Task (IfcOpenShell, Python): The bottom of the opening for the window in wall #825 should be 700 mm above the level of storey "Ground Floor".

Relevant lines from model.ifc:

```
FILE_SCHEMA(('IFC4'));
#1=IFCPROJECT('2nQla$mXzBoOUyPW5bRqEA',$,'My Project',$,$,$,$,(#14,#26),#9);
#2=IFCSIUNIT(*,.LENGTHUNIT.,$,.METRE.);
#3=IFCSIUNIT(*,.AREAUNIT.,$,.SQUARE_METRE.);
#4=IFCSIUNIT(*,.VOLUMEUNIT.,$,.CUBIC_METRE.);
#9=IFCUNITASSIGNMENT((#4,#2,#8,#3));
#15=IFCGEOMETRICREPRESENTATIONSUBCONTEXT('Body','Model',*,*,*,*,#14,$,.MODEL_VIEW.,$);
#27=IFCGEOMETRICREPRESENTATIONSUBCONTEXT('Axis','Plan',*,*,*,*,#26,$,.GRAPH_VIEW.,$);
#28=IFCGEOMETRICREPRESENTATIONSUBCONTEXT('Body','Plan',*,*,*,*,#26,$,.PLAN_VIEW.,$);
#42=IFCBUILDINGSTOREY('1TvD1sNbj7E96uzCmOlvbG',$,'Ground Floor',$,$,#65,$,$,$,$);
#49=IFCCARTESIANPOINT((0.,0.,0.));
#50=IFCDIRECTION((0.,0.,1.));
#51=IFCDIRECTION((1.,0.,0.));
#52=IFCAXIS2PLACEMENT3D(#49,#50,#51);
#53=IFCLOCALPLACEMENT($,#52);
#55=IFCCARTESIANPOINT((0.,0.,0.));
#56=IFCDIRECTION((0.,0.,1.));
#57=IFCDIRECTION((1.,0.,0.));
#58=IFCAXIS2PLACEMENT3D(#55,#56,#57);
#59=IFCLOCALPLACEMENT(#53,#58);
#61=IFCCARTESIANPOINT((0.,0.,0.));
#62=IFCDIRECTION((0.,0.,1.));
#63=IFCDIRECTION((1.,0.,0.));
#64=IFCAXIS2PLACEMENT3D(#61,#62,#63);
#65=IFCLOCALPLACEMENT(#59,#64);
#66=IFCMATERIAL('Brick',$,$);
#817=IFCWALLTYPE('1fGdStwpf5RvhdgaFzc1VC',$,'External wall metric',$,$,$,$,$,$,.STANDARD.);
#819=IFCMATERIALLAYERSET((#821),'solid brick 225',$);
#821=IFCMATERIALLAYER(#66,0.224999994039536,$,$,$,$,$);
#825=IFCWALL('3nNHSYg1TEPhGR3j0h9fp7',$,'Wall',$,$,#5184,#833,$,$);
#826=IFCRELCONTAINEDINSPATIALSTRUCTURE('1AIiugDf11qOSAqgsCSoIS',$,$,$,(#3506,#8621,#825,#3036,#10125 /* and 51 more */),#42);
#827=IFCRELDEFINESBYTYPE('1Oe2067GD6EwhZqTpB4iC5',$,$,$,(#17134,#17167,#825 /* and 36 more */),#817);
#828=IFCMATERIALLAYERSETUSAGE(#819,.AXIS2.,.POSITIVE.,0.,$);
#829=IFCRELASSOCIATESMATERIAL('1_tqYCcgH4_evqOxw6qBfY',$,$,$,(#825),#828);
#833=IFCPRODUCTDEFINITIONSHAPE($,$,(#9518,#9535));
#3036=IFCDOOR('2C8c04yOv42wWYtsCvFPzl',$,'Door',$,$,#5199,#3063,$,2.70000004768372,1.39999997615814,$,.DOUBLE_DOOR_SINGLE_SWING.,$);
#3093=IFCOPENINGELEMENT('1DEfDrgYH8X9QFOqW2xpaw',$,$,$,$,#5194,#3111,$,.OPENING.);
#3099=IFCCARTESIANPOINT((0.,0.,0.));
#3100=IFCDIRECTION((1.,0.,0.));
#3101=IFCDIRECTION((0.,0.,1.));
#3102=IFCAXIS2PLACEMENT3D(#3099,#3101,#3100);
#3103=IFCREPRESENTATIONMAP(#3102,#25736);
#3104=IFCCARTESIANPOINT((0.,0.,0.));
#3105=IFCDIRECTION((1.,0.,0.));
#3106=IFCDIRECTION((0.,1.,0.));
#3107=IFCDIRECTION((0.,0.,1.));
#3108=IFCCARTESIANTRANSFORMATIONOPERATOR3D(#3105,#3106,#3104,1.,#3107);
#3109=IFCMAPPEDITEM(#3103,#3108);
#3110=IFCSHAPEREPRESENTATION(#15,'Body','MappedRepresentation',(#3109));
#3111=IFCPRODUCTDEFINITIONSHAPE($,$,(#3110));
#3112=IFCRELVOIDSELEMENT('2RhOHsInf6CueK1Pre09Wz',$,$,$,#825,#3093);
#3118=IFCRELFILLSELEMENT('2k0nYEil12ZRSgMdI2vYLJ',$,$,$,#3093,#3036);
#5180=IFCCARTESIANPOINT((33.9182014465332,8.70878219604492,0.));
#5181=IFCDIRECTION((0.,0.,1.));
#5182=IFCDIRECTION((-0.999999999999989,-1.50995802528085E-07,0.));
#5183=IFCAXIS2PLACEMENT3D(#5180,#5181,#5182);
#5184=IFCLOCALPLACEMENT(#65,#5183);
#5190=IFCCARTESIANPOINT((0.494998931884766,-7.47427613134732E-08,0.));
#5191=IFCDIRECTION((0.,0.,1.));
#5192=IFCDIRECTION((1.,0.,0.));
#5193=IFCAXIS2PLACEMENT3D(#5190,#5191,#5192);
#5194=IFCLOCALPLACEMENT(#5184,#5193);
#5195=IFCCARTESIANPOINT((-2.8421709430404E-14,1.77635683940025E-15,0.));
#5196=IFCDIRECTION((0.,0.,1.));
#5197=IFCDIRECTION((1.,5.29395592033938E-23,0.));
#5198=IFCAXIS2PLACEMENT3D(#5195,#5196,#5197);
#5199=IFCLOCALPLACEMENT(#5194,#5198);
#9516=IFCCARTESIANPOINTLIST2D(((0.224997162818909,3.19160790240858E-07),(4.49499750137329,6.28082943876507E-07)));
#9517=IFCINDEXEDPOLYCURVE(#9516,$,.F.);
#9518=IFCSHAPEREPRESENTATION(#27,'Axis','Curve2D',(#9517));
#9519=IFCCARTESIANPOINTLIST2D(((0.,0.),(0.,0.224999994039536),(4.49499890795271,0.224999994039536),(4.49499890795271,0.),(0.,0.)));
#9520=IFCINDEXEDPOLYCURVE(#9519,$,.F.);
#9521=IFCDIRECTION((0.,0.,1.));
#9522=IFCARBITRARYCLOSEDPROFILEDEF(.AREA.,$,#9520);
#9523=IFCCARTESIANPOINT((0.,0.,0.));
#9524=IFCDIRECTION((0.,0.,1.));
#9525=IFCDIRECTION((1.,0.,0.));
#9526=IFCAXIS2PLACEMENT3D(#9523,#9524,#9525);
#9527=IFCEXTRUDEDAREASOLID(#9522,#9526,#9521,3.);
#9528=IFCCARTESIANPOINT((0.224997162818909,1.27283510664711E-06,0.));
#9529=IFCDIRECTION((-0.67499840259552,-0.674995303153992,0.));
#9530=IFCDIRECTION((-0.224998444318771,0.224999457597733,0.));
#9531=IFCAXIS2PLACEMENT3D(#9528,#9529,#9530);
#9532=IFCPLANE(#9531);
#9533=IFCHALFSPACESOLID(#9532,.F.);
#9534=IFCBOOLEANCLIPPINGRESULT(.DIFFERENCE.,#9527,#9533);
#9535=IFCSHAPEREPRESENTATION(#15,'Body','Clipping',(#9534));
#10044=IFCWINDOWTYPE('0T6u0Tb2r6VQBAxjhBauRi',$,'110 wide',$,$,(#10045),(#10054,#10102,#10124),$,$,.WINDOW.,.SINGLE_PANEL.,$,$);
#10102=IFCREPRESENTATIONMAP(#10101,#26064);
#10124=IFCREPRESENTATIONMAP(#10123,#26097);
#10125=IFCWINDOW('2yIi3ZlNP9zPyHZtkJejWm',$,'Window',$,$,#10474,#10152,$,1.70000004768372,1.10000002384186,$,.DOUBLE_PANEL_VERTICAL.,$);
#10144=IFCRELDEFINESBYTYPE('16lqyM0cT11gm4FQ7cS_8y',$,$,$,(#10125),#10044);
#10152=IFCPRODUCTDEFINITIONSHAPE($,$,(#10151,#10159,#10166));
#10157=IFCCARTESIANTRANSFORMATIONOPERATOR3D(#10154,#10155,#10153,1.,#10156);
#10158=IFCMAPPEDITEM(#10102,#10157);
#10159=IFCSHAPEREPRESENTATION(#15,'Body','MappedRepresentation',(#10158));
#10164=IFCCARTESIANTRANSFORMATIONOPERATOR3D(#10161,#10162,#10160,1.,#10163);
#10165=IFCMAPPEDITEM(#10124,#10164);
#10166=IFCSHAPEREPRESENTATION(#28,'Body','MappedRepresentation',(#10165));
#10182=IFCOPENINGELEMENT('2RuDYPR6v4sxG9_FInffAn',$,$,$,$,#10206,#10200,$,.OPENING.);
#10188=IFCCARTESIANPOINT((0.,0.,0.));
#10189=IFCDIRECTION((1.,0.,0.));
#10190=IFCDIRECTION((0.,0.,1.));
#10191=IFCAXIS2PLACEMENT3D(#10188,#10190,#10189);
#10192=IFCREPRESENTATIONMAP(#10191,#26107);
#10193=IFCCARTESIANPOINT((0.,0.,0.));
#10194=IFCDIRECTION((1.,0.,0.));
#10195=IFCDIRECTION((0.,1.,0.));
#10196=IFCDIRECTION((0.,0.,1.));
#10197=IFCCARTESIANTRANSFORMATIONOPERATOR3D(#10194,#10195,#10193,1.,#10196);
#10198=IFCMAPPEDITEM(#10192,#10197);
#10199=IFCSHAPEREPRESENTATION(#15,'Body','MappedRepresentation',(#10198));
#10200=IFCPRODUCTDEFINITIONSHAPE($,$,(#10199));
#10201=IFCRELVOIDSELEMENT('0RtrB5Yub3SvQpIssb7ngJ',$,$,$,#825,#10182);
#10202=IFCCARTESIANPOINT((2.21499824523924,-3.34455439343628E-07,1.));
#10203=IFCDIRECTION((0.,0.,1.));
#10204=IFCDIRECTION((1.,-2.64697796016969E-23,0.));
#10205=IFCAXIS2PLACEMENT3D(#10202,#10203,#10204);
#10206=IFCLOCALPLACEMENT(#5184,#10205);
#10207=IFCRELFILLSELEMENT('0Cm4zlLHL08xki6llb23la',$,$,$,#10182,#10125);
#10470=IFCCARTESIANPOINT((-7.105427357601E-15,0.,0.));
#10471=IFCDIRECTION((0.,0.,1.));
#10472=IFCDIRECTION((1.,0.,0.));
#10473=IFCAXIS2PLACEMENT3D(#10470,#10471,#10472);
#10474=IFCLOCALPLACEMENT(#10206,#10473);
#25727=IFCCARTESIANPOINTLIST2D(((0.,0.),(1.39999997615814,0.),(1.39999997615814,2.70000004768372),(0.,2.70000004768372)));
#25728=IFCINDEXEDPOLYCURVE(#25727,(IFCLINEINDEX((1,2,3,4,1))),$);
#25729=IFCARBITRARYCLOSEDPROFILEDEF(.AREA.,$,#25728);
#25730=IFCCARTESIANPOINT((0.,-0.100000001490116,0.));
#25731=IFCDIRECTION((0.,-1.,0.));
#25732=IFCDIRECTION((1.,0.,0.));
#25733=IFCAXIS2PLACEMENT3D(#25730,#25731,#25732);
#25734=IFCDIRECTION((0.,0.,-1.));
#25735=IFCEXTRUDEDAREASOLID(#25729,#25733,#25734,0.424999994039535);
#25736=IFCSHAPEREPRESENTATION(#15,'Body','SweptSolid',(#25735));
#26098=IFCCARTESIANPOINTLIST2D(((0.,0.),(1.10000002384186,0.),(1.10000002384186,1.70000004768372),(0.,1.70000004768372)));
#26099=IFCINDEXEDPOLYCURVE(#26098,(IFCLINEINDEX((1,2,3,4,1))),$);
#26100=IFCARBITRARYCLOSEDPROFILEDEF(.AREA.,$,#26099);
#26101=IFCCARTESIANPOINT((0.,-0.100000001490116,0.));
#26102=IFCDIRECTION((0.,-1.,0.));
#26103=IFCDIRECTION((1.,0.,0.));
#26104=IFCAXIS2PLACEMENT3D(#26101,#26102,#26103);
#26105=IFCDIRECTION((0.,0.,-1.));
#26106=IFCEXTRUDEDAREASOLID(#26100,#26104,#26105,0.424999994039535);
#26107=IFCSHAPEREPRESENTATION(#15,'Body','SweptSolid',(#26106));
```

```python
import numpy as np
import ifcopenshell
import ifcopenshell.api.geometry
import ifcopenshell.geom
import ifcopenshell.util.element
import ifcopenshell.util.placement
import ifcopenshell.util.shape
import ifcopenshell.util.unit

model = ifcopenshell.open("model.ifc")
unit_scale = ifcopenshell.util.unit.calculate_unit_scale(model)

window = model.by_guid("2yIi3ZlNP9zPyHZtkJejWm")
opening = window.FillsVoids[0].RelatingOpeningElement
storey = ifcopenshell.util.element.get_container(window, ifc_class="IfcBuildingStorey")
level = ifcopenshell.util.placement.get_local_placement(storey.ObjectPlacement)[2, 3]

# The opening's origin need not be at the sill, so measure its lowest point.
shape = ifcopenshell.geom.create_shape(ifcopenshell.geom.settings(), opening)
bottom = ifcopenshell.util.shape.get_shape_bottom_elevation(shape, shape.geometry) / unit_scale
dz = level + 0.7 / unit_scale - bottom

shift = np.array([0.0, 0.0, dz])
# The window is placed relative to its opening, so it follows when the opening moves.
matrix = ifcopenshell.util.placement.get_local_placement(opening.ObjectPlacement)
matrix[:3, 3] += shift
ifcopenshell.api.geometry.edit_object_placement(
    model, product=opening, matrix=matrix, is_si=False, should_transform_children=True
)

print(f"moved by {dz * unit_scale:+.3f} m")

model.write("model_rev.ifc")
```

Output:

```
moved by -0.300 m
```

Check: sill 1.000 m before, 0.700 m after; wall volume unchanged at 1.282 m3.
